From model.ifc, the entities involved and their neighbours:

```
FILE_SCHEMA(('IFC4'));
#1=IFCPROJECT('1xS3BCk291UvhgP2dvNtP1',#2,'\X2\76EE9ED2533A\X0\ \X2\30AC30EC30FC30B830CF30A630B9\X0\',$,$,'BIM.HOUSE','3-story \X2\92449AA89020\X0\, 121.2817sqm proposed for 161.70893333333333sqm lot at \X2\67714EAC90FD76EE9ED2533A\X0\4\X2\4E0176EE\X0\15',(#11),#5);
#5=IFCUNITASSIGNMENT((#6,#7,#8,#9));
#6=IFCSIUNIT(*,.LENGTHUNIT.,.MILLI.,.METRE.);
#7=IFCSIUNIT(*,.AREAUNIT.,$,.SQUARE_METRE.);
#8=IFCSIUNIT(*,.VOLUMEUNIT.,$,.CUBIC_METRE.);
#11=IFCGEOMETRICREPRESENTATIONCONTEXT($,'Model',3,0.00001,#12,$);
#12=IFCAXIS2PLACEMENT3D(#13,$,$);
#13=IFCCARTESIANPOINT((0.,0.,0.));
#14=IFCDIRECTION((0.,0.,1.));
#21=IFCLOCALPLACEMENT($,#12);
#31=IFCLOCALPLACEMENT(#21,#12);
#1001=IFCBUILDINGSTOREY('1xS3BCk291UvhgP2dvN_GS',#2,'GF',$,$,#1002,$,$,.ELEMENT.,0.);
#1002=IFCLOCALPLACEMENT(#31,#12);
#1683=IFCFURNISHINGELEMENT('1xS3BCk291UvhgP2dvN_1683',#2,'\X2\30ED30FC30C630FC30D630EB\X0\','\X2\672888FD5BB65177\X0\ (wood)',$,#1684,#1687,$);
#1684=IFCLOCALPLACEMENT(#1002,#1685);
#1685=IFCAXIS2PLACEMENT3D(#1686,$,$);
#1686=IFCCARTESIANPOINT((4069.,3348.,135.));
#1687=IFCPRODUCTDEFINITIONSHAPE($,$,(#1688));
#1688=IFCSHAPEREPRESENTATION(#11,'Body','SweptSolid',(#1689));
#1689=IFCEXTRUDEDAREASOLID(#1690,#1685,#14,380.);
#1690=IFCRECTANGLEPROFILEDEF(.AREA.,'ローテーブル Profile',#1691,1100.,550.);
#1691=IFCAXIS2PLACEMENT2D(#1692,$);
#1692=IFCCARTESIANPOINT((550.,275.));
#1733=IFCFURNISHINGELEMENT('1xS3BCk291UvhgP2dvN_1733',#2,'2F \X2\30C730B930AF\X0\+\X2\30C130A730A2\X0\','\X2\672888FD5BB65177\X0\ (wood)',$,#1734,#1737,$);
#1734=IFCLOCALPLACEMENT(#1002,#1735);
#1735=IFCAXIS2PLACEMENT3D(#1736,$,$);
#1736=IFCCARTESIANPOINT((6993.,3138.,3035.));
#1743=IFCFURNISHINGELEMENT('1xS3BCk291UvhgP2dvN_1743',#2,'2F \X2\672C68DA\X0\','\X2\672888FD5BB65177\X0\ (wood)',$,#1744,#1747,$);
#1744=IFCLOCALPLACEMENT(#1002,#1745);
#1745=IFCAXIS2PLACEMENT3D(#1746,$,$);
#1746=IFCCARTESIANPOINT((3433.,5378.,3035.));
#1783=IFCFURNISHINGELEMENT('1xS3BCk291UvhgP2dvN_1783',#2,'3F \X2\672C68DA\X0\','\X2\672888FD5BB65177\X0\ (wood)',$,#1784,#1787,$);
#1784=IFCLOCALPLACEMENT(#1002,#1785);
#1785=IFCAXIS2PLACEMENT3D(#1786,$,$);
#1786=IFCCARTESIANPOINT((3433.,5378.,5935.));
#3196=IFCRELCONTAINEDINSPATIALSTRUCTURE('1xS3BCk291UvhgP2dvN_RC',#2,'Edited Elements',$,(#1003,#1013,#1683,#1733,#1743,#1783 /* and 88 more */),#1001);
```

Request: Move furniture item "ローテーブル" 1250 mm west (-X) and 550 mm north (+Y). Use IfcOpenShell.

```python
import ifcopenshell
import ifcopenshell.api.geometry
import ifcopenshell.util.placement

model = ifcopenshell.open("model.ifc")

item = model.by_guid("1xS3BCk291UvhgP2dvN_1683")
matrix = ifcopenshell.util.placement.get_local_placement(item.ObjectPlacement)
matrix[0, 3] -= 1250.0
matrix[1, 3] += 550.0
ifcopenshell.api.geometry.edit_object_placement(model, product=item, matrix=matrix, is_si=False)

print(ifcopenshell.util.placement.get_local_placement(item.ObjectPlacement).round(3) + 0.0)

model.write("model_v2.ifc")
```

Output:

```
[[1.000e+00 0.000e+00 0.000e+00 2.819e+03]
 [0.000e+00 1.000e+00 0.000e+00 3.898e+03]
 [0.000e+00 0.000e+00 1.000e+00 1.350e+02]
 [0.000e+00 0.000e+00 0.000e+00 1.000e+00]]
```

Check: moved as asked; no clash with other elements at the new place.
